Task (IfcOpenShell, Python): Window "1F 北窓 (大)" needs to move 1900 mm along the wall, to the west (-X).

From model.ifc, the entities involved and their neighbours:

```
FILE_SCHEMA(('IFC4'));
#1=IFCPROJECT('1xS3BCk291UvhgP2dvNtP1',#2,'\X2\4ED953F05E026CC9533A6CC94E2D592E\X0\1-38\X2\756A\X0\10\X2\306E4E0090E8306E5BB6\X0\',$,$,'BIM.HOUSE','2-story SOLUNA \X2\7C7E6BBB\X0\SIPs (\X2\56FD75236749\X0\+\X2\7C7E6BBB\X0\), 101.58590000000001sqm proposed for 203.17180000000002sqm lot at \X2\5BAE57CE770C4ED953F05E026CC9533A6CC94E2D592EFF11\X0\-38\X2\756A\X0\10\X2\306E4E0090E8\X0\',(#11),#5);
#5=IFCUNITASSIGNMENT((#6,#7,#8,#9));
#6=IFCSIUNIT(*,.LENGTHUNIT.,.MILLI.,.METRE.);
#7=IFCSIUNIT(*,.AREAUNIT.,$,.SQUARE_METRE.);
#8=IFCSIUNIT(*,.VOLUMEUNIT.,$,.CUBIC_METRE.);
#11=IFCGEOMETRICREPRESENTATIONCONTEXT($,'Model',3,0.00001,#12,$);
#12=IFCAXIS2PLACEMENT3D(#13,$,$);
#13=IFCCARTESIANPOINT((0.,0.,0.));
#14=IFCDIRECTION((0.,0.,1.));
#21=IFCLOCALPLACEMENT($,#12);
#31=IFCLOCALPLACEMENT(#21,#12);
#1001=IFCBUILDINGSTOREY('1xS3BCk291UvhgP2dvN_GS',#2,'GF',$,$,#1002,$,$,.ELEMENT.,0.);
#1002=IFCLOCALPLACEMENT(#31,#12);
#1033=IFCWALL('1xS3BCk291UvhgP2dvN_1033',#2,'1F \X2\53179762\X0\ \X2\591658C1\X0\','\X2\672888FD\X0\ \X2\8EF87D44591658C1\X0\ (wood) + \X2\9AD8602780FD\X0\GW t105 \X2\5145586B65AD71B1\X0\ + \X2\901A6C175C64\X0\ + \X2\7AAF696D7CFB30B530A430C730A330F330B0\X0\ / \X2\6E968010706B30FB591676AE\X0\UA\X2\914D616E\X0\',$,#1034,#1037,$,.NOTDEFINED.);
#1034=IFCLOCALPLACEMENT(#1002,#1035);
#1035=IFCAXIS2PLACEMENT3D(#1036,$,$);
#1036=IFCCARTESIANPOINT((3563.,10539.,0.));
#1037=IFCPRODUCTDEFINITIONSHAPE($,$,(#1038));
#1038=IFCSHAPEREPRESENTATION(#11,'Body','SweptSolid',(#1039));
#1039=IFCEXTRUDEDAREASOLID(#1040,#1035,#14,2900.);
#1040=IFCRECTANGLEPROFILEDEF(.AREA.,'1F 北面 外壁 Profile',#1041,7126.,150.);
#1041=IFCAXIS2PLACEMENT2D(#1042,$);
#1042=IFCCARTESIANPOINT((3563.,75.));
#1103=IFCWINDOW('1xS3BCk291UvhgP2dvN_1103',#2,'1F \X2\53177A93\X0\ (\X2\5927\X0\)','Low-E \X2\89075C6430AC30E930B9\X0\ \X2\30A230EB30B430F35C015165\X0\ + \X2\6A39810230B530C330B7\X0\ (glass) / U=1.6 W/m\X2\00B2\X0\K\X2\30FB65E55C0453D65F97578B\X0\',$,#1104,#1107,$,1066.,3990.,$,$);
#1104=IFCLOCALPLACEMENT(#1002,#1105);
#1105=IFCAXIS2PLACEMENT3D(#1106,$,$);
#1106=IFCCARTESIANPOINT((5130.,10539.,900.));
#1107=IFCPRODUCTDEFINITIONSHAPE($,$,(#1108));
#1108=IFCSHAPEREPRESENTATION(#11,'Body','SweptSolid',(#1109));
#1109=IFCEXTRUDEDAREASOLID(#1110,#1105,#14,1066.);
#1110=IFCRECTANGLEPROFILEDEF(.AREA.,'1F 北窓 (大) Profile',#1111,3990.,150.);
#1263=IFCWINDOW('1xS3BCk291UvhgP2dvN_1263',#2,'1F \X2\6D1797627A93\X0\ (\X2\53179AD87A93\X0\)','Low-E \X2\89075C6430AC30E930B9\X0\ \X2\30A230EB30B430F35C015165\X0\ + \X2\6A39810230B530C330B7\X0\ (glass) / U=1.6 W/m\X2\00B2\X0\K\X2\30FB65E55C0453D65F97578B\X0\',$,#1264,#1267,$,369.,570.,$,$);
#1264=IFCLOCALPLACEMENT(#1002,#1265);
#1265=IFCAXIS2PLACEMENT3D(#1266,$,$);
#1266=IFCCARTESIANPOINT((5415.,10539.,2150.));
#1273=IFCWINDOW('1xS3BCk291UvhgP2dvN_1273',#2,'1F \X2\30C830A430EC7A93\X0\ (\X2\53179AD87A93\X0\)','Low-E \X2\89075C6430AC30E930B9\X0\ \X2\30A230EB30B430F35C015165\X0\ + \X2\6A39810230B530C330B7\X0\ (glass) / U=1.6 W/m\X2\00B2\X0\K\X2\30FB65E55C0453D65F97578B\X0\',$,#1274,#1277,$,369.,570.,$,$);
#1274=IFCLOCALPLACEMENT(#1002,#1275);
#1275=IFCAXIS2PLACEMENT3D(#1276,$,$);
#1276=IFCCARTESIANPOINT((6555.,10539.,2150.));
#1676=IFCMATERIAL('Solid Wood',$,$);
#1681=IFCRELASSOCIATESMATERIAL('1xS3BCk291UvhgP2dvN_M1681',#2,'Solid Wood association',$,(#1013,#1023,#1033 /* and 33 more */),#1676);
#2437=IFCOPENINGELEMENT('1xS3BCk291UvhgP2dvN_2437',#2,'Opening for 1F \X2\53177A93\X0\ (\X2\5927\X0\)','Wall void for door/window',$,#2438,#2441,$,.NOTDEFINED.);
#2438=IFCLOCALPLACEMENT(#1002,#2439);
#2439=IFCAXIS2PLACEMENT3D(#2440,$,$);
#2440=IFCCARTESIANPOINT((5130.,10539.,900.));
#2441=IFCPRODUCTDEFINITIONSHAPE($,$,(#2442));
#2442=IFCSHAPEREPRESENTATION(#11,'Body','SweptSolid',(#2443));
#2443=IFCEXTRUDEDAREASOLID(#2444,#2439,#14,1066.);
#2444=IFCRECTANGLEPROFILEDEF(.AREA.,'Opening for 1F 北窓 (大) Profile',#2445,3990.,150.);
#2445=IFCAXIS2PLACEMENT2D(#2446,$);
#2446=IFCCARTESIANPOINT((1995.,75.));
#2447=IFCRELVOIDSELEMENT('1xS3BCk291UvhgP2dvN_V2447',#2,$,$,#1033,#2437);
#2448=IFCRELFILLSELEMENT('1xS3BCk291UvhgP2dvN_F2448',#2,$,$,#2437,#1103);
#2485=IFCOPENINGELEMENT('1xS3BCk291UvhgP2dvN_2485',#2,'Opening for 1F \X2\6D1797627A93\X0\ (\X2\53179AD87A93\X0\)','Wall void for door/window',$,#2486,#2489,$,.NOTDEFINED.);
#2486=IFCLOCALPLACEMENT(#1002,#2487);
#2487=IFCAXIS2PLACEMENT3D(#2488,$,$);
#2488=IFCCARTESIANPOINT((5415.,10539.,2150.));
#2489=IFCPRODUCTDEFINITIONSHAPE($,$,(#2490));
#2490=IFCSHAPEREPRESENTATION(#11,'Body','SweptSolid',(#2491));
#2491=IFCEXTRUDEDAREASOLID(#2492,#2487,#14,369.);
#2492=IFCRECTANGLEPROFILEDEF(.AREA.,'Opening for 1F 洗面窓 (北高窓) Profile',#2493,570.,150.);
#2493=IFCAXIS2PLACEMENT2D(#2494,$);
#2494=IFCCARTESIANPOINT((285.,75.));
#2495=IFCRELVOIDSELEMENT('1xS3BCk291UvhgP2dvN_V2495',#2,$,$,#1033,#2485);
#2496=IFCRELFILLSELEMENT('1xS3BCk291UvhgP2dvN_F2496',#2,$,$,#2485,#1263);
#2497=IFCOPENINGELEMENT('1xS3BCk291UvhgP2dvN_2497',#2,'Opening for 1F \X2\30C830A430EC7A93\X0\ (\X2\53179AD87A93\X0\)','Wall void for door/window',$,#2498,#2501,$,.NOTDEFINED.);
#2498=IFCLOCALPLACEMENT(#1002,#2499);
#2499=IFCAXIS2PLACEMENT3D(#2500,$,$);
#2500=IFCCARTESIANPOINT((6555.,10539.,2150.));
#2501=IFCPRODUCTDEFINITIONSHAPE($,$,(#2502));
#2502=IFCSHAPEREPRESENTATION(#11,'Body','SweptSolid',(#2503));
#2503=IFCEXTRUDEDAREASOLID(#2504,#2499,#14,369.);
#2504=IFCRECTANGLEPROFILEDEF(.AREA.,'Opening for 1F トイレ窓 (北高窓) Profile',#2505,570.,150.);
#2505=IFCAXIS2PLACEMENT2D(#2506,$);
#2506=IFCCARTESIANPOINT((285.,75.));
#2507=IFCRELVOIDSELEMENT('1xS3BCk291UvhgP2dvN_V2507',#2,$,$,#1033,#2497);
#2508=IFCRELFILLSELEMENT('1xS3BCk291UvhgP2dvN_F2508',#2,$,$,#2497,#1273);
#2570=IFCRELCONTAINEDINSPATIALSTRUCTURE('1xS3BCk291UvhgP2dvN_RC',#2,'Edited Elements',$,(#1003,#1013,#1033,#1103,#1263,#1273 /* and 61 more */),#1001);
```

```python
import ifcopenshell
import ifcopenshell.api.geometry
import ifcopenshell.util.placement
import ifcopenshell.util.unit

model = ifcopenshell.open("model.ifc")
unit_scale = ifcopenshell.util.unit.calculate_unit_scale(model)

window = model.by_id(1103)
opening = window.FillsVoids[0].RelatingOpeningElement
wall = opening.VoidsElements[0].RelatingBuildingElement

wall_matrix = ifcopenshell.util.placement.get_local_placement(wall.ObjectPlacement)
shift = wall_matrix[:3, 0] * -1.9 / unit_scale
before = ifcopenshell.util.placement.get_local_placement(window.ObjectPlacement)[:3, 3].copy()

# The window is not placed relative to its opening, so move both.
for product in (opening, window):
    matrix = ifcopenshell.util.placement.get_local_placement(product.ObjectPlacement)
    matrix[:3, 3] += shift
    ifcopenshell.api.geometry.edit_object_placement(model, product=product, matrix=matrix, is_si=False)

after = ifcopenshell.util.placement.get_local_placement(window.ObjectPlacement)[:3, 3]
print("window moved by", (after - before).round(3) + 0.0)

model.write("model_rev.ifc")
```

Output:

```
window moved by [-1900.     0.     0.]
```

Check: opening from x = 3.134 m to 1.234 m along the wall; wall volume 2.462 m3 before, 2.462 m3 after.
